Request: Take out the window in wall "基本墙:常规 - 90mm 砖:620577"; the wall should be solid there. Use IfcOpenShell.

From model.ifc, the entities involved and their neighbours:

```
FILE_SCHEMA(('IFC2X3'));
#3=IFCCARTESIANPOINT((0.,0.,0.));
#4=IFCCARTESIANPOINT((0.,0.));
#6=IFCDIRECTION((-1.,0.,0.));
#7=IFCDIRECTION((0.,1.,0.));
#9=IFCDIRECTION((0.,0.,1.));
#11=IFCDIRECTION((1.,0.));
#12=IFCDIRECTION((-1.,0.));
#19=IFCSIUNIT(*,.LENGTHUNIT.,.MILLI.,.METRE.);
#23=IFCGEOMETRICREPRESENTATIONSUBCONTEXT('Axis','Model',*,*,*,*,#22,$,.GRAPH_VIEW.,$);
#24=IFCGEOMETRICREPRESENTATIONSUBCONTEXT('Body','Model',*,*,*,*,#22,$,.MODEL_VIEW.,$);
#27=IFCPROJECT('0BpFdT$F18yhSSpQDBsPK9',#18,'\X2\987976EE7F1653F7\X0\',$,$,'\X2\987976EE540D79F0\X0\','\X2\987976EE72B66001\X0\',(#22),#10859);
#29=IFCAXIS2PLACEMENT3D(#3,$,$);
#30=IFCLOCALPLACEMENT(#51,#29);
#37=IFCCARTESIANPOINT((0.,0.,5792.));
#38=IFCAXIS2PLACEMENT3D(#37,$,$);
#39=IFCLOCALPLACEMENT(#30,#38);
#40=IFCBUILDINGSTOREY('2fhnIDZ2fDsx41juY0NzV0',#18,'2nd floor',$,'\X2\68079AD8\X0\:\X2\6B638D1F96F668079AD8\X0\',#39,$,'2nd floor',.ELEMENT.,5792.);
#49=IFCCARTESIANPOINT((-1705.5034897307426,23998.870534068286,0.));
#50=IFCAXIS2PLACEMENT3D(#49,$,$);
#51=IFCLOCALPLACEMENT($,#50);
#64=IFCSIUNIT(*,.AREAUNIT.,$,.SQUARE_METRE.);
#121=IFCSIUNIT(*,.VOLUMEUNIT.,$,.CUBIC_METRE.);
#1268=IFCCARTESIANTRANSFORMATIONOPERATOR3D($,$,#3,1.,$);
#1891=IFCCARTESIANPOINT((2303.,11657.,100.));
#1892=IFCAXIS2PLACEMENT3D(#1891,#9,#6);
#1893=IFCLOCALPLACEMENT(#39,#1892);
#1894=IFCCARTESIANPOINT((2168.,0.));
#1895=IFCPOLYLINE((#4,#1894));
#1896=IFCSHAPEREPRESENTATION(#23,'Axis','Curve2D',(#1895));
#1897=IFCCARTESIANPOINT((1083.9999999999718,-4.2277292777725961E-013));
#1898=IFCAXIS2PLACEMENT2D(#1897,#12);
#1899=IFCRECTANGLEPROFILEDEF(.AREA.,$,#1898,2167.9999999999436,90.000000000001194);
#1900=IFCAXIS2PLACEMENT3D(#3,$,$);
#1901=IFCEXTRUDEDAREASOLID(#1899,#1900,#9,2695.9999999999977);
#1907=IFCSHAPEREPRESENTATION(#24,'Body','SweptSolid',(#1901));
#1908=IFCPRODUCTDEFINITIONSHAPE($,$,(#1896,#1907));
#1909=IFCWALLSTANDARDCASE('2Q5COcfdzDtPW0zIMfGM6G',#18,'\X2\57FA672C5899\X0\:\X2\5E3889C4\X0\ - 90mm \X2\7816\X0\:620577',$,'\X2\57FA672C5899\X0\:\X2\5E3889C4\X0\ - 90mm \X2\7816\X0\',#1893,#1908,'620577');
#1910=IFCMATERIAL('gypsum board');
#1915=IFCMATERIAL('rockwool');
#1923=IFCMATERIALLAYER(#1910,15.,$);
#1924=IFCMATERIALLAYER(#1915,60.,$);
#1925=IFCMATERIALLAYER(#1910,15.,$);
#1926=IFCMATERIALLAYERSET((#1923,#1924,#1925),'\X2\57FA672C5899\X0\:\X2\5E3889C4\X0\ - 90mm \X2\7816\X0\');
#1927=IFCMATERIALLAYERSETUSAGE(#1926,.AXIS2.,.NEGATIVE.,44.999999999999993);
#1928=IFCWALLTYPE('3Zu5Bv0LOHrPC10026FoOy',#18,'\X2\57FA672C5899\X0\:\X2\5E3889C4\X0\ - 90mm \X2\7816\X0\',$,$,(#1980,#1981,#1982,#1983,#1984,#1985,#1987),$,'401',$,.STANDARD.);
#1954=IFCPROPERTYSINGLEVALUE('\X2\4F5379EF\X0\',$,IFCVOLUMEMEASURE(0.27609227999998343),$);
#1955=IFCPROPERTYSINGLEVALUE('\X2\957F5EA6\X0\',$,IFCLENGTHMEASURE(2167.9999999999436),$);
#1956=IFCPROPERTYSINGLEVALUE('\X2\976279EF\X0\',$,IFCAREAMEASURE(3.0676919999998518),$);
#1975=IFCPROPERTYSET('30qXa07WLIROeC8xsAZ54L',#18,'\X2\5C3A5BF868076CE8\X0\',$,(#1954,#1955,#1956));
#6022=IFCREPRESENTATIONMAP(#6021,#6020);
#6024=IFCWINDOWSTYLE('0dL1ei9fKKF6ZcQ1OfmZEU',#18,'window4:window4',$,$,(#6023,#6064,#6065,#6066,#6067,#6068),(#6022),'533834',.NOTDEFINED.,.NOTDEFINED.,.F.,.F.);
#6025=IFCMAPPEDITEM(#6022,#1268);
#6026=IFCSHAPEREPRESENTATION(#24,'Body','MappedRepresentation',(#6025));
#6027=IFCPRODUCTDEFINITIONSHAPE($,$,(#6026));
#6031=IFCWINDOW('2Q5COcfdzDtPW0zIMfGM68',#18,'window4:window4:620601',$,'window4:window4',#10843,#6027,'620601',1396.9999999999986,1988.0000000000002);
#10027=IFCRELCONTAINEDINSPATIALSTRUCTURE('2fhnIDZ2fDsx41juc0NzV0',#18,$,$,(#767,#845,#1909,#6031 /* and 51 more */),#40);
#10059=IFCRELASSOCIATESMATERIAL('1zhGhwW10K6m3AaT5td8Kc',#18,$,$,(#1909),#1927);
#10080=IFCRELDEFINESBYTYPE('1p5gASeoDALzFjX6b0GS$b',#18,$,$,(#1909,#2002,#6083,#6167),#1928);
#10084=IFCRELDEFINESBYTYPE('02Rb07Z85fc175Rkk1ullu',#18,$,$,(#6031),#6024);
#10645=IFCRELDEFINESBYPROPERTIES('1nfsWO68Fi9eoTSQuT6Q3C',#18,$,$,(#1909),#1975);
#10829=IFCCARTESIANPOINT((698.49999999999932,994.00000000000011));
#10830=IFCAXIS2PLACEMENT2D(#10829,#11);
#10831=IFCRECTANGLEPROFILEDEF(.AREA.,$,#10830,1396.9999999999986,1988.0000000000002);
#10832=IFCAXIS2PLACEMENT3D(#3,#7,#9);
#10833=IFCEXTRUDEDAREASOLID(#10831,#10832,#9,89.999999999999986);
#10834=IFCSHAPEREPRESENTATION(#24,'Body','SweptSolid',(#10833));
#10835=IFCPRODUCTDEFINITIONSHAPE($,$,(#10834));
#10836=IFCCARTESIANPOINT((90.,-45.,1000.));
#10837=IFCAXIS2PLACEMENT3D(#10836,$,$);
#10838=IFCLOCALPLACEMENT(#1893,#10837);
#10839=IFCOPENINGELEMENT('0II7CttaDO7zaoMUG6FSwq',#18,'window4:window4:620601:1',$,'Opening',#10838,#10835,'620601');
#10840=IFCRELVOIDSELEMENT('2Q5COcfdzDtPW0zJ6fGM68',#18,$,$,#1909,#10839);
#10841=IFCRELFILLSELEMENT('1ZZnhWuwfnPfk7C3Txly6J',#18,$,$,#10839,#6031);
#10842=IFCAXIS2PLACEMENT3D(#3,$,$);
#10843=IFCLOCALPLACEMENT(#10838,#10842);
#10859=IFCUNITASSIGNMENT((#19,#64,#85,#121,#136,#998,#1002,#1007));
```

```python
import ifcopenshell
import ifcopenshell.api.feature
import ifcopenshell.api.pset
import ifcopenshell.api.root
import ifcopenshell.geom
import ifcopenshell.util.element
import ifcopenshell.util.shape
import ifcopenshell.util.unit

model = ifcopenshell.open("model.ifc")
area_scale = ifcopenshell.util.unit.calculate_unit_scale(model, "AREAUNIT")
volume_scale = ifcopenshell.util.unit.calculate_unit_scale(model, "VOLUMEUNIT")
settings = ifcopenshell.geom.settings()


def volume(element):
    """Net volume in cubic metres, openings subtracted."""
    shape = ifcopenshell.geom.create_shape(settings, element)
    return ifcopenshell.util.shape.get_volume(shape.geometry)


window = model.by_guid("2Q5COcfdzDtPW0zIMfGM68")
opening = window.FillsVoids[0].RelatingOpeningElement
wall = opening.VoidsElements[0].RelatingBuildingElement
before = volume(wall)

ifcopenshell.api.root.remove_product(model, product=window)
ifcopenshell.api.feature.remove_feature(model, feature=opening)

after = volume(wall)
thickness = 0.09  # wall thickness in metres

# Update the wall's stored quantities.
pset = model.by_id(ifcopenshell.util.element.get_pset(wall, "尺寸标注", should_inherit=False)["id"])
ifcopenshell.api.pset.edit_pset(model, pset=pset, properties={
    "体积": model.create_entity("IfcVolumeMeasure", after / volume_scale),
    "面积": model.create_entity("IfcAreaMeasure", after / thickness / area_scale),
})

print(f"wall volume {before:.3f} -> {after:.3f} m3")

model.write("model-out.ifc")
```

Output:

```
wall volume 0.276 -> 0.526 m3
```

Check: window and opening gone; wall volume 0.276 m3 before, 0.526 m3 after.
